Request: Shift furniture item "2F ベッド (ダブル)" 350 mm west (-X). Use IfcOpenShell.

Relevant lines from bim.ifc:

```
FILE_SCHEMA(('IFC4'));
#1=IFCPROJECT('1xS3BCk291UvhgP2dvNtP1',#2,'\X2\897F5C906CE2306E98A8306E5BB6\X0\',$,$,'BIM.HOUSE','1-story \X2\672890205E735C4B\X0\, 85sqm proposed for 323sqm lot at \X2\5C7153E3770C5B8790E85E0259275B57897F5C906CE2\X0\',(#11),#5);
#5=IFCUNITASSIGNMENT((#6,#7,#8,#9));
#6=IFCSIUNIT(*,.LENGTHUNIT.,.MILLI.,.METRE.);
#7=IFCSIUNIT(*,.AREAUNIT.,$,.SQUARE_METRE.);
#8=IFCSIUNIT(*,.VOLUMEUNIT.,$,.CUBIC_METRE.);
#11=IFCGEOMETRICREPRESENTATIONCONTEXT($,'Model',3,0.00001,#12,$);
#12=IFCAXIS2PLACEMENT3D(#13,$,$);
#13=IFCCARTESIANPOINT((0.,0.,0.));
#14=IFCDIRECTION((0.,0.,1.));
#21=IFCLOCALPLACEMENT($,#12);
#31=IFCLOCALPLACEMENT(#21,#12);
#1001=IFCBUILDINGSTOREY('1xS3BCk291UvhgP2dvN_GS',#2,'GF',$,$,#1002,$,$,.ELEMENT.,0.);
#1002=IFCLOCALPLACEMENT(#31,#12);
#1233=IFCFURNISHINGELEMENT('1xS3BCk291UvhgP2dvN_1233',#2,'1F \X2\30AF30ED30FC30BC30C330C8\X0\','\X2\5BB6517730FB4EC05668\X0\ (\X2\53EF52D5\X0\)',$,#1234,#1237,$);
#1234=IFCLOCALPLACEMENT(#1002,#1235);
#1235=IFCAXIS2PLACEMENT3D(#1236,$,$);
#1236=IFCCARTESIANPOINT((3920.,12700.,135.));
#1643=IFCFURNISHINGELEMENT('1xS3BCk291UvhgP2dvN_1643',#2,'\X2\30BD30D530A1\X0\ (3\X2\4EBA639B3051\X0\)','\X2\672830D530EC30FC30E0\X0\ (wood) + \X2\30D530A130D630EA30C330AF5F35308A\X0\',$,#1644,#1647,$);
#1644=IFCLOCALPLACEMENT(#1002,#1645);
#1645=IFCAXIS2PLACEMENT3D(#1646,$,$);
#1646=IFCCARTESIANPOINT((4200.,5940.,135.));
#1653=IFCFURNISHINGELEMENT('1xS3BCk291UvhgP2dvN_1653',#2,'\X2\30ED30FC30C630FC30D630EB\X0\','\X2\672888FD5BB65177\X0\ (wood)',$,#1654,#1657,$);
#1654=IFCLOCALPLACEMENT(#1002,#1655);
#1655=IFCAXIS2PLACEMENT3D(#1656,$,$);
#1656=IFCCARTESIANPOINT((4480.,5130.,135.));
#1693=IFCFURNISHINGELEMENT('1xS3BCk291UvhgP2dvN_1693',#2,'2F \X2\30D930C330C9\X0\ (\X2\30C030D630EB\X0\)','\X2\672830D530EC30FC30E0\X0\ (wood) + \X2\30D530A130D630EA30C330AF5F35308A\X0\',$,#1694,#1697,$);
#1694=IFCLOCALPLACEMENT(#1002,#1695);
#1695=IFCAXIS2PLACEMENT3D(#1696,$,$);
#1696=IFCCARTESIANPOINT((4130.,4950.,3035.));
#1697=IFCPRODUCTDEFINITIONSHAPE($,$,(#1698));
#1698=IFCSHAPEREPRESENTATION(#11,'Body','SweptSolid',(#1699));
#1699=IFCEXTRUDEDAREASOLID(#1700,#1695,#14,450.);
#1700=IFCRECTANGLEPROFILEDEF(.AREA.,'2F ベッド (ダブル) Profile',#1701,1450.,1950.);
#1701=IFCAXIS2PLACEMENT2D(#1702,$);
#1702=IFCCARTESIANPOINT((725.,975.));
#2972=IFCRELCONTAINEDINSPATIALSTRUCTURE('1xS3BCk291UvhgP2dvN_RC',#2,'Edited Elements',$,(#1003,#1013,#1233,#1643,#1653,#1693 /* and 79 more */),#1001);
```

```python
import ifcopenshell
import ifcopenshell.api.geometry
import ifcopenshell.util.placement
import ifcopenshell.util.unit

model = ifcopenshell.open("bim.ifc")
unit_scale = ifcopenshell.util.unit.calculate_unit_scale(model)

item = model.by_guid("1xS3BCk291UvhgP2dvN_1693")
matrix = ifcopenshell.util.placement.get_local_placement(item.ObjectPlacement)
matrix[0, 3] -= 0.35 / unit_scale
ifcopenshell.api.geometry.edit_object_placement(model, product=item, matrix=matrix, is_si=False)

print(ifcopenshell.util.placement.get_local_placement(item.ObjectPlacement).round(3) + 0.0)

model.write("bim_v2.ifc")
```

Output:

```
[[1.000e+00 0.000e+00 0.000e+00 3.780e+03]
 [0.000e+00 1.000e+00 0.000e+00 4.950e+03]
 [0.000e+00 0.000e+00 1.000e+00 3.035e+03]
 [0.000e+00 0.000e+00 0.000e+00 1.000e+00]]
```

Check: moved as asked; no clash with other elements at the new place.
